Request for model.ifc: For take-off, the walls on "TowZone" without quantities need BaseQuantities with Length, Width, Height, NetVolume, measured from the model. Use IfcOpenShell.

First a look at what the model holds.

```python
import ifcopenshell
import ifcopenshell.util.element
import ifcopenshell.util.unit

model = ifcopenshell.open("model.ifc")
print(model.schema)
for unit_type in ("LENGTHUNIT", "AREAUNIT", "VOLUMEUNIT"):
    print(unit_type, ifcopenshell.util.unit.calculate_unit_scale(model, unit_type))
storey = next(s for s in model.by_type("IfcBuildingStorey") if s.Name == "TowZone")
walls = [e for e in ifcopenshell.util.element.get_decomposition(storey) if e.is_a("IfcWall")]
for e in sorted(walls, key=lambda e: e.id()):
    print(e.id(), e.is_a(), e.Name, list(ifcopenshell.util.element.get_psets(e, qtos_only=True)), sep=" | ")
```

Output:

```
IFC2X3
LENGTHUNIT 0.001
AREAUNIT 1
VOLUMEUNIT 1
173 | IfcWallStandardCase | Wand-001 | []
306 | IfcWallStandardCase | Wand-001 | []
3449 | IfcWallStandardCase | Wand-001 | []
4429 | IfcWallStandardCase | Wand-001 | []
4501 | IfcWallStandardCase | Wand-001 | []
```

```python
import ifcopenshell
import ifcopenshell.api.pset
import ifcopenshell.geom
import ifcopenshell.util.element
import ifcopenshell.util.shape
import ifcopenshell.util.unit

model = ifcopenshell.open("model.ifc")
unit_scale = ifcopenshell.util.unit.calculate_unit_scale(model)
volume_scale = ifcopenshell.util.unit.calculate_unit_scale(model, "VOLUMEUNIT")
settings = ifcopenshell.geom.settings()

storey = next(s for s in model.by_type("IfcBuildingStorey") if s.Name == "TowZone")
walls = [e for e in ifcopenshell.util.element.get_decomposition(storey) if e.is_a("IfcWall")]

for e in sorted(walls, key=lambda e: e.id()):
    if ifcopenshell.util.element.get_psets(e, qtos_only=True, should_inherit=False):
        continue
    # Geometry comes back in metres, in the element's own axes.
    shape = ifcopenshell.geom.create_shape(settings, e)
    values = {
        "Length": ifcopenshell.util.shape.get_x(shape.geometry) / unit_scale,
        "Width": ifcopenshell.util.shape.get_y(shape.geometry) / unit_scale,
        "Height": ifcopenshell.util.shape.get_z(shape.geometry) / unit_scale,
        "NetVolume": ifcopenshell.util.shape.get_volume(shape.geometry) / volume_scale,
    }
    qto = ifcopenshell.api.pset.add_qto(model, product=e, name="BaseQuantities")
    ifcopenshell.api.pset.edit_qto(model, qto=qto, properties=values)
    print(e.id(), {k: round(v, 3) for k, v in values.items()})

model.write("model_v2.ifc")
```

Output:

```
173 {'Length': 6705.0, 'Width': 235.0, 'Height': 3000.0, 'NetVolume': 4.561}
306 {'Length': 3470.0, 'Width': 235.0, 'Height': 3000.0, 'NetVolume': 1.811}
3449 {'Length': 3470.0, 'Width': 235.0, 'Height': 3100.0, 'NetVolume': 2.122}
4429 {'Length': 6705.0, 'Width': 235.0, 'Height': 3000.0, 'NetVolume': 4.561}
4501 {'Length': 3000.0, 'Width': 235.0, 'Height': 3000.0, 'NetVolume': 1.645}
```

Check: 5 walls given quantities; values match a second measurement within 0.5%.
